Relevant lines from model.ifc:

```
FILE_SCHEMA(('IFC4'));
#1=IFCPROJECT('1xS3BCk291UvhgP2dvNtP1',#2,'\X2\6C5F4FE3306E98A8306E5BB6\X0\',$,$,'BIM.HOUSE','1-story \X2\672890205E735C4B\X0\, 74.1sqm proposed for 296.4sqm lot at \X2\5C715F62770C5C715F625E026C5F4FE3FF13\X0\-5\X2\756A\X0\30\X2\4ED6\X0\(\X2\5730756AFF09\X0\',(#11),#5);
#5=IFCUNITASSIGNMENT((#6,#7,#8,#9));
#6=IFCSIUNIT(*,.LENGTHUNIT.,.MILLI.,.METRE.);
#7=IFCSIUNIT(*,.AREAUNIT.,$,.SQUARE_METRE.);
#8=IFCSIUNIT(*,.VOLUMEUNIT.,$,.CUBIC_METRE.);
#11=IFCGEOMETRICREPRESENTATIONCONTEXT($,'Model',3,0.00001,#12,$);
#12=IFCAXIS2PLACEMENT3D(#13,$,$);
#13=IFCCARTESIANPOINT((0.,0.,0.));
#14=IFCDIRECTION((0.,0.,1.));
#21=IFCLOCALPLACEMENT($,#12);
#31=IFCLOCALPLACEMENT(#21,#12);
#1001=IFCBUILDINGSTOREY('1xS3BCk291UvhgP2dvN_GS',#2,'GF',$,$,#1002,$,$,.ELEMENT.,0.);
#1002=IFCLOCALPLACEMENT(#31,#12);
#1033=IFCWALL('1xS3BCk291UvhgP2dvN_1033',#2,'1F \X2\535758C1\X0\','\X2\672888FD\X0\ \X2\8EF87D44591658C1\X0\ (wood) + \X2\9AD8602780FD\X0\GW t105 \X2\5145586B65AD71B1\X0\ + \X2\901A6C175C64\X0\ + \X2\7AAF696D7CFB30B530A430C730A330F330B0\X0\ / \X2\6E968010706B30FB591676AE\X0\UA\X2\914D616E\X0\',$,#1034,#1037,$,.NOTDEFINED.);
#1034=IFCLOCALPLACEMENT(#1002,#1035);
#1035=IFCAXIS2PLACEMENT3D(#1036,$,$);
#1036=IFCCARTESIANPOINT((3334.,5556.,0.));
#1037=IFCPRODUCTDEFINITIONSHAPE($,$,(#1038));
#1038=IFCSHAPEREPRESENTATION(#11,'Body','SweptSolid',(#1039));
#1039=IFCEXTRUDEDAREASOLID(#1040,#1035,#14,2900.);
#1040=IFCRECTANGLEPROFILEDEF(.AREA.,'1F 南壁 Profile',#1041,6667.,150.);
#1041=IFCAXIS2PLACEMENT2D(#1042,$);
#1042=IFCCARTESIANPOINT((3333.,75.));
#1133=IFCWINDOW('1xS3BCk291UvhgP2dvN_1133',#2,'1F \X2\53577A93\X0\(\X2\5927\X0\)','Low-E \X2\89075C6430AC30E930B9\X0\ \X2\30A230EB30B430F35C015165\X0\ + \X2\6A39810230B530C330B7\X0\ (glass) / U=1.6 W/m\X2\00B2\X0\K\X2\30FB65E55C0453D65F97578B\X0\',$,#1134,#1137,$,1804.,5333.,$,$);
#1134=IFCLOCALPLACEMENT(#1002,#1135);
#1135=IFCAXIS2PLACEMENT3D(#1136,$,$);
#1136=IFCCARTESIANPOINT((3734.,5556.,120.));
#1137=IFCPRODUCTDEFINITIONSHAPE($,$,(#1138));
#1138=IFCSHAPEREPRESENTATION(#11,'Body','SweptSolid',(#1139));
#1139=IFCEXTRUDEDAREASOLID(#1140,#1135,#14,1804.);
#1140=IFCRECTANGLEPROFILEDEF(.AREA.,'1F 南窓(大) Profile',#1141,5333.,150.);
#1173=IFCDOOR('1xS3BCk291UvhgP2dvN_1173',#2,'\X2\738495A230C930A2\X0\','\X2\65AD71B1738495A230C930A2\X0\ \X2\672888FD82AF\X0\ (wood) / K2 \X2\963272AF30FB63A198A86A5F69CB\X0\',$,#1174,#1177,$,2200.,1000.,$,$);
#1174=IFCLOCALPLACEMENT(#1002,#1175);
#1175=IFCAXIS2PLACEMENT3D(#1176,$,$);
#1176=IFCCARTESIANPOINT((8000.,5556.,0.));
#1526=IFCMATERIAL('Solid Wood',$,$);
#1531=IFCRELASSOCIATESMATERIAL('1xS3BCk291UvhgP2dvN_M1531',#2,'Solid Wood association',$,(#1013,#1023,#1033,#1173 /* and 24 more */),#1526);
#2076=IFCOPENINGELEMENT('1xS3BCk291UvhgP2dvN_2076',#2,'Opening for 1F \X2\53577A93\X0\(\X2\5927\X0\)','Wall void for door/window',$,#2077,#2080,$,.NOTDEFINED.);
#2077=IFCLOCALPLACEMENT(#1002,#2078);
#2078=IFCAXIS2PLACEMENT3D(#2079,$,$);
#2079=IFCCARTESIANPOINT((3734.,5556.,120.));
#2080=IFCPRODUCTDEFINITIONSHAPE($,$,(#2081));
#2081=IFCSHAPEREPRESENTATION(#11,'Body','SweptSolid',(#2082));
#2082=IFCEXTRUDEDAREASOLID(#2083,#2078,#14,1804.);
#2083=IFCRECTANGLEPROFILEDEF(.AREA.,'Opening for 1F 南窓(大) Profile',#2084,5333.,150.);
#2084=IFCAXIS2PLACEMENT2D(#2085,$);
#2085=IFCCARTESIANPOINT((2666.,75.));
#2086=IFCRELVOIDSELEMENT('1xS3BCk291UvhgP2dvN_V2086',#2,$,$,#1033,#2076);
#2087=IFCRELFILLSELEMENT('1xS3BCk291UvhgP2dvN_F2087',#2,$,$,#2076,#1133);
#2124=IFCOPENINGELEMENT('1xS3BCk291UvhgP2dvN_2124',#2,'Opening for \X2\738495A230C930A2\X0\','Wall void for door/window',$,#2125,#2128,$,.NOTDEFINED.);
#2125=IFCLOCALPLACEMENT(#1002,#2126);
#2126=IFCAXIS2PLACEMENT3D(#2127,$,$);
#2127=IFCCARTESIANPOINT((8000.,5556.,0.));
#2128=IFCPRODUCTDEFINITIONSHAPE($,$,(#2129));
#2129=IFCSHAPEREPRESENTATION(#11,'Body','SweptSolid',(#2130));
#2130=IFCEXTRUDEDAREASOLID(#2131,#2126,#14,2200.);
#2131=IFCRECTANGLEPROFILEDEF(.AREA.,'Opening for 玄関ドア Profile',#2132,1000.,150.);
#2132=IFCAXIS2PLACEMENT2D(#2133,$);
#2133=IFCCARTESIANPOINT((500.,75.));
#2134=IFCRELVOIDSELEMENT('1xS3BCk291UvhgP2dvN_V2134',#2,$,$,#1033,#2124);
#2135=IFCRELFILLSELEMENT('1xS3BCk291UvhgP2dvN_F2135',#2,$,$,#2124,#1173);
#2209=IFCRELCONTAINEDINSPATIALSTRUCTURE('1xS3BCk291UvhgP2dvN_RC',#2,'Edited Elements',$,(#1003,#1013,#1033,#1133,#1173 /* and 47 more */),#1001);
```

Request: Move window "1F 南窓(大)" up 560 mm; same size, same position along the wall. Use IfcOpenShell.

```python
import numpy as np
import ifcopenshell
import ifcopenshell.api.geometry
import ifcopenshell.util.placement
import ifcopenshell.util.unit

model = ifcopenshell.open("model.ifc")
unit_scale = ifcopenshell.util.unit.calculate_unit_scale(model)

window = model.by_guid("1xS3BCk291UvhgP2dvN_1133")
opening = window.FillsVoids[0].RelatingOpeningElement
dz = 560.0

shift = np.array([0.0, 0.0, dz])
# The window is not placed relative to its opening, so move both.
for product in (opening, window):
    matrix = ifcopenshell.util.placement.get_local_placement(product.ObjectPlacement)
    matrix[:3, 3] += shift
    ifcopenshell.api.geometry.edit_object_placement(model, product=product, matrix=matrix, is_si=False)

print(f"moved by {dz * unit_scale:+.3f} m")

model.write("model_edited.ifc")
```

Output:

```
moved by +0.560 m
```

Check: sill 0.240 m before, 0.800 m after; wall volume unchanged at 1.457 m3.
